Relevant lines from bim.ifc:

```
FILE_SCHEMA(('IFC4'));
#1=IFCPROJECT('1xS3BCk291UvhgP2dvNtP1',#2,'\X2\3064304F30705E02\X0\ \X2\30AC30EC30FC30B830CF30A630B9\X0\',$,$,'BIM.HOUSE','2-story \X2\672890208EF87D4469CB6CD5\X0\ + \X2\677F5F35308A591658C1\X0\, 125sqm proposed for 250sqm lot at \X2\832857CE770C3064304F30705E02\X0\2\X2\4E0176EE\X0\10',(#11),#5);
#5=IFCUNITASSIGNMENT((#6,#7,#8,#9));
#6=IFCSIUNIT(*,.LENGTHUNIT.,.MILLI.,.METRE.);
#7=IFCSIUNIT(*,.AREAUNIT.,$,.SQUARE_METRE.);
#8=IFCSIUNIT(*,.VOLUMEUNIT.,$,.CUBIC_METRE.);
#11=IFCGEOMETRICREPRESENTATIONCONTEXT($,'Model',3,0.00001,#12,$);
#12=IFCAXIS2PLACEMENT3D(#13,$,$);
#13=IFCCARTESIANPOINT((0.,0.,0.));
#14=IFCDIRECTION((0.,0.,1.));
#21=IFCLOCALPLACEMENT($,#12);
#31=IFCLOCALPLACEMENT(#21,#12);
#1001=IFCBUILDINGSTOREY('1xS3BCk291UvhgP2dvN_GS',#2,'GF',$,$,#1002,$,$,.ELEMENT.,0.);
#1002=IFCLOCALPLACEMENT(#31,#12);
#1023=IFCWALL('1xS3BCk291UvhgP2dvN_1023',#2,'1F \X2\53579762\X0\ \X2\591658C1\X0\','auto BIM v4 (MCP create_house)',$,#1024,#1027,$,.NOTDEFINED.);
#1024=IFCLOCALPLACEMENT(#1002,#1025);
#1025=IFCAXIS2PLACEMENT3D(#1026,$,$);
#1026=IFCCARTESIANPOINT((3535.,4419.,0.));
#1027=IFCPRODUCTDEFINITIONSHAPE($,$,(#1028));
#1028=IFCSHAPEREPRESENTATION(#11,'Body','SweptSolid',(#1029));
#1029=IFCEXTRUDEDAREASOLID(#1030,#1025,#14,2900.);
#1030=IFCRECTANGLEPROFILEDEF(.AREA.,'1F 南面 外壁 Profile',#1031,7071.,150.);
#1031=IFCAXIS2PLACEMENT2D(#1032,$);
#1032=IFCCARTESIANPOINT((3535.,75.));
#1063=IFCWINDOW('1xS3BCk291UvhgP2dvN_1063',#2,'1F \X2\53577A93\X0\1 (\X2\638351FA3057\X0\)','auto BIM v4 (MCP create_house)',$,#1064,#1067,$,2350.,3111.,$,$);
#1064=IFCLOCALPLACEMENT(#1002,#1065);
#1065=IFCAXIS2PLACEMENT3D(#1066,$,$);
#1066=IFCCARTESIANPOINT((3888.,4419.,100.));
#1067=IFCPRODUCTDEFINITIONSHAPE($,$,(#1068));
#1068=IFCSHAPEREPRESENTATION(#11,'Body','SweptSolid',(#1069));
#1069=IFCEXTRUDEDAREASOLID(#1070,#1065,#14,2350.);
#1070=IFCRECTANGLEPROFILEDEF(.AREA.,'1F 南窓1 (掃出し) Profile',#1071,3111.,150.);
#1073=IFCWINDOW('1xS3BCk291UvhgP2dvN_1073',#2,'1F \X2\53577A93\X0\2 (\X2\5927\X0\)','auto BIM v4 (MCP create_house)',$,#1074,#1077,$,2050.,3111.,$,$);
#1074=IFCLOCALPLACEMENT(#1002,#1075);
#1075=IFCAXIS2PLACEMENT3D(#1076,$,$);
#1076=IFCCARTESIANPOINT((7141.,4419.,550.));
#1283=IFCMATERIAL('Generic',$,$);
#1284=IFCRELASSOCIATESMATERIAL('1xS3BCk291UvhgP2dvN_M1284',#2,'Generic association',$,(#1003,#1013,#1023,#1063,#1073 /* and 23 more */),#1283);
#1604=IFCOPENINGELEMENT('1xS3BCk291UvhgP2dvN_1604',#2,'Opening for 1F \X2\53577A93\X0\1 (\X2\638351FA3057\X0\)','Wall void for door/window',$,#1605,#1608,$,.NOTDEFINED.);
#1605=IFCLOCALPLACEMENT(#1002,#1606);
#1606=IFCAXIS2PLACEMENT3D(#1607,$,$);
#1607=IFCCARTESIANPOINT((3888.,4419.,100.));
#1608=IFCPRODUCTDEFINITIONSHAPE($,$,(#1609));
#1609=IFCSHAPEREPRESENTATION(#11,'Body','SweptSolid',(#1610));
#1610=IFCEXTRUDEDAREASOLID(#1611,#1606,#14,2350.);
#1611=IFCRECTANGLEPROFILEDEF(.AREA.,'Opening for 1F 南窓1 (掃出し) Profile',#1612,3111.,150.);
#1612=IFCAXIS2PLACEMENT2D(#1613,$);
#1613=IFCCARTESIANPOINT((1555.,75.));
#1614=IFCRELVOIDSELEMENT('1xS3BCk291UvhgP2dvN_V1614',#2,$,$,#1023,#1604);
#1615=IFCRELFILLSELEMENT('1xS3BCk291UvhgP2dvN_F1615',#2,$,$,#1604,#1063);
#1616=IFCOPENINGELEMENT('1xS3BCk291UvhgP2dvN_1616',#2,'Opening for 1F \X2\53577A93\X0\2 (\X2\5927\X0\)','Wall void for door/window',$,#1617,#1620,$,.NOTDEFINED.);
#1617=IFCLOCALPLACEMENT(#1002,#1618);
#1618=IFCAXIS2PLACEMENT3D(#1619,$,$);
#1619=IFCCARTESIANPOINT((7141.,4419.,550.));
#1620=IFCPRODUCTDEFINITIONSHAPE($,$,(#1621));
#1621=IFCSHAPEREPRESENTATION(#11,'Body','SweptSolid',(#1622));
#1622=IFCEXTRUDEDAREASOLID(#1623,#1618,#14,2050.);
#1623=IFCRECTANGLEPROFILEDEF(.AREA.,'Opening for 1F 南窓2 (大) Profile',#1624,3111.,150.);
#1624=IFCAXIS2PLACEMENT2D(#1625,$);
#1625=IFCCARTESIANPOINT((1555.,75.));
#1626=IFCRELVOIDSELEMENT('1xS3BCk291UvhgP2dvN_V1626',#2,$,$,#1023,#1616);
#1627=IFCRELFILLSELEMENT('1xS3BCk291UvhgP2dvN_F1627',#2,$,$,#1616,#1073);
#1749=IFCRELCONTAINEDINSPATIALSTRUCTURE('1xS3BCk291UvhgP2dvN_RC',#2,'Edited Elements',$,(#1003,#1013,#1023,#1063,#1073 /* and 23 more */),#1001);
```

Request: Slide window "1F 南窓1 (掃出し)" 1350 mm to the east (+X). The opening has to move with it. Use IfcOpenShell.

```python
import ifcopenshell
import ifcopenshell.api.geometry
import ifcopenshell.util.placement

model = ifcopenshell.open("bim.ifc")

window = model.by_id(1063)
opening = window.FillsVoids[0].RelatingOpeningElement
wall = opening.VoidsElements[0].RelatingBuildingElement

wall_matrix = ifcopenshell.util.placement.get_local_placement(wall.ObjectPlacement)
shift = wall_matrix[:3, 0] * 1350.0
before = ifcopenshell.util.placement.get_local_placement(window.ObjectPlacement)[:3, 3].copy()

# The window is not placed relative to its opening, so move both.
for product in (opening, window):
    matrix = ifcopenshell.util.placement.get_local_placement(product.ObjectPlacement)
    matrix[:3, 3] += shift
    ifcopenshell.api.geometry.edit_object_placement(model, product=product, matrix=matrix, is_si=False)

after = ifcopenshell.util.placement.get_local_placement(window.ObjectPlacement)[:3, 3]
print("window moved by", (after - before).round(3) + 0.0)

model.write("bim_v2.ifc")
```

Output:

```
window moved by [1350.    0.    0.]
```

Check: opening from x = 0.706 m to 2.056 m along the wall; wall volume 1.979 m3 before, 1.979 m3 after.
